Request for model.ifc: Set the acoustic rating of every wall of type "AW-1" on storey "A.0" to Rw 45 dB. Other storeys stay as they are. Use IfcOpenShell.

First a look at what the model holds.

```python
import ifcopenshell
import ifcopenshell.util.element

model = ifcopenshell.open("model.ifc")
print(model.schema)
storey = next(s for s in model.by_type("IfcBuildingStorey") if s.Name == "A.0")
walls = [e for e in ifcopenshell.util.element.get_decomposition(storey) if e.is_a("IfcWall")]
seen = {}
for e in walls:
    element_type = ifcopenshell.util.element.get_type(e)
    key = (element_type.Name if element_type != e and element_type else None, ifcopenshell.util.element.get_pset(e, "Pset_WallCommon", "AcousticRating"))
    seen[key] = seen.get(key, 0) + 1
for (name, value), count in sorted(seen.items(), key=str):
    print(count, "x", name, "|", value)
```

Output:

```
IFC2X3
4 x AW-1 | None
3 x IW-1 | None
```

```python
import ifcopenshell
import ifcopenshell.api.pset
import ifcopenshell.util.element

model = ifcopenshell.open("model.ifc")

storey = next(s for s in model.by_type("IfcBuildingStorey") if s.Name == "A.0")
walls = [e for e in ifcopenshell.util.element.get_decomposition(storey) if e.is_a("IfcWall")]

count = 0
for e in walls:
    element_type = ifcopenshell.util.element.get_type(e)
    if element_type in (None, e) or element_type.Name != "AW-1":
        continue
    # add_pset returns the element's existing set when there is one.
    pset = ifcopenshell.api.pset.add_pset(model, product=e, name="Pset_WallCommon")
    ifcopenshell.api.pset.edit_pset(model, pset=pset, properties={"AcousticRating": "Rw 45 dB"})
    count += 1

print(count, "walls updated")

model.write("model_v2.ifc")
```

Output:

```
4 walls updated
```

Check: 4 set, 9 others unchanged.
